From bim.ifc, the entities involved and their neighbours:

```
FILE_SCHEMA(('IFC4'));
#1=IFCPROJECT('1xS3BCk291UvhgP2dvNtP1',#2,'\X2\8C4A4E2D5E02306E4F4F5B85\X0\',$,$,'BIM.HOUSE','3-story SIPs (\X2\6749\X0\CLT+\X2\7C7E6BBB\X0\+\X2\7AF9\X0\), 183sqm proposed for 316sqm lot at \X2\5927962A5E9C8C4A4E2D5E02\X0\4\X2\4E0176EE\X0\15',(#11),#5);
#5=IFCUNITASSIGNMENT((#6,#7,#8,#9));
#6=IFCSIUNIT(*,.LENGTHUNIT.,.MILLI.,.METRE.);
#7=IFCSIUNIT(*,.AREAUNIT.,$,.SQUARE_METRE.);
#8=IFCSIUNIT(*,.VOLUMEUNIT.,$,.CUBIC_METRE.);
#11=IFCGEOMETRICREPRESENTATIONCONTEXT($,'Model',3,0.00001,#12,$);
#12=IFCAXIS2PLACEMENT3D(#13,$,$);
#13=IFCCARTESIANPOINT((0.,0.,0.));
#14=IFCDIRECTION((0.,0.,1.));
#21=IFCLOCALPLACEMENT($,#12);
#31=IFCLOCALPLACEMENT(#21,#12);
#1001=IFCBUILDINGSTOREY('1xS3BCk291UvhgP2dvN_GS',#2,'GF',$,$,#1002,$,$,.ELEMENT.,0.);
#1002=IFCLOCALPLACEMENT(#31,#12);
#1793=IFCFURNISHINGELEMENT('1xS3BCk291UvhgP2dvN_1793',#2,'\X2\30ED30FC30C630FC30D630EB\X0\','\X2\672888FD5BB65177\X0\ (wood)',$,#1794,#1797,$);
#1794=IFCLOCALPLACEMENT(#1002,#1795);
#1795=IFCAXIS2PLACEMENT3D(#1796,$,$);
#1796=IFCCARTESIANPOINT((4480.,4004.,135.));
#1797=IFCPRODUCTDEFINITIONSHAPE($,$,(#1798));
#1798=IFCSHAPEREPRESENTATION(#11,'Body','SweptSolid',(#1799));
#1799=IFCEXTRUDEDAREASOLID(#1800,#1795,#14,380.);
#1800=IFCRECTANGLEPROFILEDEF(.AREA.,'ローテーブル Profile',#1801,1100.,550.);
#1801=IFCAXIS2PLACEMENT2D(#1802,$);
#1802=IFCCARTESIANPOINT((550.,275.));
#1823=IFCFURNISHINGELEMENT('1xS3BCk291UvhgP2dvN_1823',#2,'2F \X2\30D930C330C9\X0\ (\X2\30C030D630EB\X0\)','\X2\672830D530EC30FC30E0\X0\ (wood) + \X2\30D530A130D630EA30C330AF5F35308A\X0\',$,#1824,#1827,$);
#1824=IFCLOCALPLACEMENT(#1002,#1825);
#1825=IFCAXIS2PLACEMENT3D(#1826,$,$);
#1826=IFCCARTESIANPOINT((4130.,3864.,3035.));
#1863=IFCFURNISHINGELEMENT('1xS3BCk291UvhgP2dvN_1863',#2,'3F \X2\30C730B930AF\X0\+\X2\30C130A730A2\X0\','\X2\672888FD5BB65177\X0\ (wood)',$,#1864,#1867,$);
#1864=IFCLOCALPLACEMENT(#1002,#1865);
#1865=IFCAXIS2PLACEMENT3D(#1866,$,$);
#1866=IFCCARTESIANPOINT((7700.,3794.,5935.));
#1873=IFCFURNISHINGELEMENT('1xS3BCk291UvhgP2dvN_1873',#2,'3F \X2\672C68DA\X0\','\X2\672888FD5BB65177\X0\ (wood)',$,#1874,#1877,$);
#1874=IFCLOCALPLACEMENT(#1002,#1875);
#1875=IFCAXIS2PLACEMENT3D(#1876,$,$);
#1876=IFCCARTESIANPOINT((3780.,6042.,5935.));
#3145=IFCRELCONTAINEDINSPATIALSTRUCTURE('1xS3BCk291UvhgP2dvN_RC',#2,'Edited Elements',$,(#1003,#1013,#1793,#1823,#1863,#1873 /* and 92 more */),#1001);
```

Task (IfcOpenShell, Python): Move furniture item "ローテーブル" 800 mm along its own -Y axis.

```python
import ifcopenshell
import ifcopenshell.api.geometry
import ifcopenshell.util.placement

model = ifcopenshell.open("bim.ifc")

item = model.by_guid("1xS3BCk291UvhgP2dvN_1793")
matrix = ifcopenshell.util.placement.get_local_placement(item.ObjectPlacement)
matrix[:3, 3] -= matrix[:3, 1] * 800.0
ifcopenshell.api.geometry.edit_object_placement(model, product=item, matrix=matrix, is_si=False)

print(ifcopenshell.util.placement.get_local_placement(item.ObjectPlacement).round(3) + 0.0)

model.write("bim_v2.ifc")
```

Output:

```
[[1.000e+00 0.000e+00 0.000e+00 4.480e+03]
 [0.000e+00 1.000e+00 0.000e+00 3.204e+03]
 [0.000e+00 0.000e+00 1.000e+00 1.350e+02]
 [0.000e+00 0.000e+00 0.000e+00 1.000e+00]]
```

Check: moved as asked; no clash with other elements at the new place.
